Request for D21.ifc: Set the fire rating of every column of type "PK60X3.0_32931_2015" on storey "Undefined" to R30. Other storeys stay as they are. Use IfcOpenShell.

First a look at what the model holds.

```python
import ifcopenshell
import ifcopenshell.util.element

model = ifcopenshell.open("D21.ifc")
print(model.schema)
storey = next(s for s in model.by_type("IfcBuildingStorey") if s.Name == "Undefined")
columns = [e for e in ifcopenshell.util.element.get_decomposition(storey) if e.is_a("IfcColumn")]
seen = {}
for e in columns:
    element_type = ifcopenshell.util.element.get_type(e)
    key = (element_type.Name if element_type != e and element_type else None, ifcopenshell.util.element.get_pset(e, "Pset_ColumnCommon", "FireRating"))
    seen[key] = seen.get(key, 0) + 1
for (name, value), count in sorted(seen.items(), key=str):
    print(count, "x", name, "|", value)
```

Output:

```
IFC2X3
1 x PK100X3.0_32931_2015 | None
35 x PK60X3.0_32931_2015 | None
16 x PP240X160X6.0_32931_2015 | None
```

```python
import ifcopenshell
import ifcopenshell.api.pset
import ifcopenshell.util.element

model = ifcopenshell.open("D21.ifc")

storey = next(s for s in model.by_type("IfcBuildingStorey") if s.Name == "Undefined")
columns = [e for e in ifcopenshell.util.element.get_decomposition(storey) if e.is_a("IfcColumn")]

count = 0
for e in columns:
    element_type = ifcopenshell.util.element.get_type(e)
    if element_type in (None, e) or element_type.Name != "PK60X3.0_32931_2015":
        continue
    found = ifcopenshell.util.element.get_pset(e, "Pset_ColumnCommon", should_inherit=False)
    if found:
        pset = model.by_id(found["id"])
        if len(ifcopenshell.util.element.get_elements_by_pset(pset)) > 1:
            pset = ifcopenshell.api.pset.unshare_pset(model, products=[e], pset=pset)[0]
    else:
        pset = ifcopenshell.api.pset.add_pset(model, product=e, name="Pset_ColumnCommon")
    ifcopenshell.api.pset.edit_pset(model, pset=pset, properties={"FireRating": "R30"})
    count += 1

print(count, "columns updated")

model.write("D21_edited.ifc")
```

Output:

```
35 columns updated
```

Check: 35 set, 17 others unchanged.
